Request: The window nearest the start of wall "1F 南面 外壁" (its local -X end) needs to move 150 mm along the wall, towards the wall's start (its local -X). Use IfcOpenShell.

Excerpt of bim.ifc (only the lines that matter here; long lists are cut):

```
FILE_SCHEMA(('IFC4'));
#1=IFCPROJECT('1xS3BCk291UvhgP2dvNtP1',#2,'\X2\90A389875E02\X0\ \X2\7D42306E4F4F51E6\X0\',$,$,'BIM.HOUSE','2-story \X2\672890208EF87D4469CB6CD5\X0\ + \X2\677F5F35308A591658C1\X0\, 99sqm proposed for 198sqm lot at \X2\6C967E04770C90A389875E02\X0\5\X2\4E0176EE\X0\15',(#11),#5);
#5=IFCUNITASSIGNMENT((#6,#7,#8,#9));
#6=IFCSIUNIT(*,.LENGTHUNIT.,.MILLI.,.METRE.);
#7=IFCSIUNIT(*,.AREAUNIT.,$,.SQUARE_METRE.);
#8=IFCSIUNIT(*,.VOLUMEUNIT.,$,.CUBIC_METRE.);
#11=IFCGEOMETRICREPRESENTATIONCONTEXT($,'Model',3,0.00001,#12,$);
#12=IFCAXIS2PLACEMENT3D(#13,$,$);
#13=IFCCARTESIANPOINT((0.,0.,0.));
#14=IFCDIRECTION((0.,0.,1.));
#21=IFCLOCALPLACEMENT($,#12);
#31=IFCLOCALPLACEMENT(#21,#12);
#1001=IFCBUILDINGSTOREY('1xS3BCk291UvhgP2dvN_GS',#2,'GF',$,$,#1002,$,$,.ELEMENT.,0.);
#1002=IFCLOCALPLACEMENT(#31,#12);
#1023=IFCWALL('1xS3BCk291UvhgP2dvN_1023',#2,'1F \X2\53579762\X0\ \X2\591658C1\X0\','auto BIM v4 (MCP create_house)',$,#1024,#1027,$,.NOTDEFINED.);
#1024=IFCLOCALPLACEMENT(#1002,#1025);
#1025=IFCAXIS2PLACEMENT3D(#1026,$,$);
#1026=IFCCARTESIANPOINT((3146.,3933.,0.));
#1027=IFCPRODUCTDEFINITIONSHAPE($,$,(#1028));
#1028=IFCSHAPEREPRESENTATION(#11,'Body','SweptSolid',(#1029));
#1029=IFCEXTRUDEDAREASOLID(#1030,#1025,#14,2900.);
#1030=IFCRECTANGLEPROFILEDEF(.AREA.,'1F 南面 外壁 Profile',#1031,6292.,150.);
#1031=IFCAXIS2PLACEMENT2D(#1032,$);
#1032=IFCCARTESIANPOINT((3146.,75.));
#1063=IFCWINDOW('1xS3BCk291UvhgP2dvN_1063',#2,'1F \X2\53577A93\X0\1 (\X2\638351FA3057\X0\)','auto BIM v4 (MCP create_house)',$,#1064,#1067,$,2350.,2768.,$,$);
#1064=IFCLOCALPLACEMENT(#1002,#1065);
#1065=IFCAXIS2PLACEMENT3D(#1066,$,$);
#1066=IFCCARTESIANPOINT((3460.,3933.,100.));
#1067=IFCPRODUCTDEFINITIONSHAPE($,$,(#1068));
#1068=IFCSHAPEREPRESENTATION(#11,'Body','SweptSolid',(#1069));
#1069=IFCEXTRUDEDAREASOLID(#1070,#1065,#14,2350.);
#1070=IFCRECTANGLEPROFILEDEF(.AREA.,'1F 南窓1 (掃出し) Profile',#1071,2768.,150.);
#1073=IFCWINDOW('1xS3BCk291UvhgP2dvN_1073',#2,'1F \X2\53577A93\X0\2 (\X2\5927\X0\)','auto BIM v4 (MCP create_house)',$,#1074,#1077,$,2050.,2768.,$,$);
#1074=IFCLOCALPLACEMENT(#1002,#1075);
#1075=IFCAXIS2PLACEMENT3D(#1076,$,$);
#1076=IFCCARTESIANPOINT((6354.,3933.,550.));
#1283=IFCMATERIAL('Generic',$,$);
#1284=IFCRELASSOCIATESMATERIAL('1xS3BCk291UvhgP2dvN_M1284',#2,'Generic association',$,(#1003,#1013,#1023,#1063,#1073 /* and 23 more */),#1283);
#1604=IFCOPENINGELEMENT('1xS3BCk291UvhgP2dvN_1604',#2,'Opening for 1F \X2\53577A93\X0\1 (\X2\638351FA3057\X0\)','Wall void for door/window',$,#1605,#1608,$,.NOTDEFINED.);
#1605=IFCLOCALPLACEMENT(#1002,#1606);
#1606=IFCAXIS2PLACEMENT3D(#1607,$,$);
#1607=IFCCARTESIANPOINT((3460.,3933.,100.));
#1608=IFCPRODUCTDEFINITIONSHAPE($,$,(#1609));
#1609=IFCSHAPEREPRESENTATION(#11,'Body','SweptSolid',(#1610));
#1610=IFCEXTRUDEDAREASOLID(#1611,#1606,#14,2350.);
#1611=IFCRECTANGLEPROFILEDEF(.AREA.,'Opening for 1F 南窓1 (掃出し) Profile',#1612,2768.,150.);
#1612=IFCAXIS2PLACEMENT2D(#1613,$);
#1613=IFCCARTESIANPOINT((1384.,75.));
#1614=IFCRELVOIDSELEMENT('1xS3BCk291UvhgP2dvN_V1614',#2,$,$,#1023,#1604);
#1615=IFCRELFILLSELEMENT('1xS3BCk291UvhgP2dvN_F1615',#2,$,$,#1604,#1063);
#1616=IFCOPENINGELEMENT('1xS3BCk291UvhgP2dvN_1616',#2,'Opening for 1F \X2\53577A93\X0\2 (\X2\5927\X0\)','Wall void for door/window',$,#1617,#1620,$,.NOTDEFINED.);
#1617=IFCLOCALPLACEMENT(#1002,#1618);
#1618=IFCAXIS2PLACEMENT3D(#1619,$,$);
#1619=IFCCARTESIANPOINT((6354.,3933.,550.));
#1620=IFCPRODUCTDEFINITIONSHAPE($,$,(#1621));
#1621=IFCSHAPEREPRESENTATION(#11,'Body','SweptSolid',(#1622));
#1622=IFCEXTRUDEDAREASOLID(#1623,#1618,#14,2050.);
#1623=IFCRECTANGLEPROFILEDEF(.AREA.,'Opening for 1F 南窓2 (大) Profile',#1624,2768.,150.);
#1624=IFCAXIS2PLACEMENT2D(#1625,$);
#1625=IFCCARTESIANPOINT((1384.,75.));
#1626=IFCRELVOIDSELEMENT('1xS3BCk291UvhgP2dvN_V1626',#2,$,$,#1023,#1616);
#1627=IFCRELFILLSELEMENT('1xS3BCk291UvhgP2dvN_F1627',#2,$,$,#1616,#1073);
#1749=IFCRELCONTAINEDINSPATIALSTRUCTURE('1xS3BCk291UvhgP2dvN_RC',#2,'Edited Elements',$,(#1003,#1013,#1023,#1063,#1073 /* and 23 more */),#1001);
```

```python
import ifcopenshell
import ifcopenshell.api.geometry
import ifcopenshell.util.placement
import ifcopenshell.util.unit

model = ifcopenshell.open("bim.ifc")
unit_scale = ifcopenshell.util.unit.calculate_unit_scale(model)

window = model.by_id(1063)
opening = window.FillsVoids[0].RelatingOpeningElement
wall = opening.VoidsElements[0].RelatingBuildingElement

wall_matrix = ifcopenshell.util.placement.get_local_placement(wall.ObjectPlacement)
shift = wall_matrix[:3, 0] * -0.15 / unit_scale
before = ifcopenshell.util.placement.get_local_placement(window.ObjectPlacement)[:3, 3].copy()

# The window is not placed relative to its opening, so move both.
for product in (opening, window):
    matrix = ifcopenshell.util.placement.get_local_placement(product.ObjectPlacement)
    matrix[:3, 3] += shift
    ifcopenshell.api.geometry.edit_object_placement(model, product=product, matrix=matrix, is_si=False)

after = ifcopenshell.util.placement.get_local_placement(window.ObjectPlacement)[:3, 3]
print("window moved by", (after - before).round(3) + 0.0)

model.write("bim_v2.ifc")
```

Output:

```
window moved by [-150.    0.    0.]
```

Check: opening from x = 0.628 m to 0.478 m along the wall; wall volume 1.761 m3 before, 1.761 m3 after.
